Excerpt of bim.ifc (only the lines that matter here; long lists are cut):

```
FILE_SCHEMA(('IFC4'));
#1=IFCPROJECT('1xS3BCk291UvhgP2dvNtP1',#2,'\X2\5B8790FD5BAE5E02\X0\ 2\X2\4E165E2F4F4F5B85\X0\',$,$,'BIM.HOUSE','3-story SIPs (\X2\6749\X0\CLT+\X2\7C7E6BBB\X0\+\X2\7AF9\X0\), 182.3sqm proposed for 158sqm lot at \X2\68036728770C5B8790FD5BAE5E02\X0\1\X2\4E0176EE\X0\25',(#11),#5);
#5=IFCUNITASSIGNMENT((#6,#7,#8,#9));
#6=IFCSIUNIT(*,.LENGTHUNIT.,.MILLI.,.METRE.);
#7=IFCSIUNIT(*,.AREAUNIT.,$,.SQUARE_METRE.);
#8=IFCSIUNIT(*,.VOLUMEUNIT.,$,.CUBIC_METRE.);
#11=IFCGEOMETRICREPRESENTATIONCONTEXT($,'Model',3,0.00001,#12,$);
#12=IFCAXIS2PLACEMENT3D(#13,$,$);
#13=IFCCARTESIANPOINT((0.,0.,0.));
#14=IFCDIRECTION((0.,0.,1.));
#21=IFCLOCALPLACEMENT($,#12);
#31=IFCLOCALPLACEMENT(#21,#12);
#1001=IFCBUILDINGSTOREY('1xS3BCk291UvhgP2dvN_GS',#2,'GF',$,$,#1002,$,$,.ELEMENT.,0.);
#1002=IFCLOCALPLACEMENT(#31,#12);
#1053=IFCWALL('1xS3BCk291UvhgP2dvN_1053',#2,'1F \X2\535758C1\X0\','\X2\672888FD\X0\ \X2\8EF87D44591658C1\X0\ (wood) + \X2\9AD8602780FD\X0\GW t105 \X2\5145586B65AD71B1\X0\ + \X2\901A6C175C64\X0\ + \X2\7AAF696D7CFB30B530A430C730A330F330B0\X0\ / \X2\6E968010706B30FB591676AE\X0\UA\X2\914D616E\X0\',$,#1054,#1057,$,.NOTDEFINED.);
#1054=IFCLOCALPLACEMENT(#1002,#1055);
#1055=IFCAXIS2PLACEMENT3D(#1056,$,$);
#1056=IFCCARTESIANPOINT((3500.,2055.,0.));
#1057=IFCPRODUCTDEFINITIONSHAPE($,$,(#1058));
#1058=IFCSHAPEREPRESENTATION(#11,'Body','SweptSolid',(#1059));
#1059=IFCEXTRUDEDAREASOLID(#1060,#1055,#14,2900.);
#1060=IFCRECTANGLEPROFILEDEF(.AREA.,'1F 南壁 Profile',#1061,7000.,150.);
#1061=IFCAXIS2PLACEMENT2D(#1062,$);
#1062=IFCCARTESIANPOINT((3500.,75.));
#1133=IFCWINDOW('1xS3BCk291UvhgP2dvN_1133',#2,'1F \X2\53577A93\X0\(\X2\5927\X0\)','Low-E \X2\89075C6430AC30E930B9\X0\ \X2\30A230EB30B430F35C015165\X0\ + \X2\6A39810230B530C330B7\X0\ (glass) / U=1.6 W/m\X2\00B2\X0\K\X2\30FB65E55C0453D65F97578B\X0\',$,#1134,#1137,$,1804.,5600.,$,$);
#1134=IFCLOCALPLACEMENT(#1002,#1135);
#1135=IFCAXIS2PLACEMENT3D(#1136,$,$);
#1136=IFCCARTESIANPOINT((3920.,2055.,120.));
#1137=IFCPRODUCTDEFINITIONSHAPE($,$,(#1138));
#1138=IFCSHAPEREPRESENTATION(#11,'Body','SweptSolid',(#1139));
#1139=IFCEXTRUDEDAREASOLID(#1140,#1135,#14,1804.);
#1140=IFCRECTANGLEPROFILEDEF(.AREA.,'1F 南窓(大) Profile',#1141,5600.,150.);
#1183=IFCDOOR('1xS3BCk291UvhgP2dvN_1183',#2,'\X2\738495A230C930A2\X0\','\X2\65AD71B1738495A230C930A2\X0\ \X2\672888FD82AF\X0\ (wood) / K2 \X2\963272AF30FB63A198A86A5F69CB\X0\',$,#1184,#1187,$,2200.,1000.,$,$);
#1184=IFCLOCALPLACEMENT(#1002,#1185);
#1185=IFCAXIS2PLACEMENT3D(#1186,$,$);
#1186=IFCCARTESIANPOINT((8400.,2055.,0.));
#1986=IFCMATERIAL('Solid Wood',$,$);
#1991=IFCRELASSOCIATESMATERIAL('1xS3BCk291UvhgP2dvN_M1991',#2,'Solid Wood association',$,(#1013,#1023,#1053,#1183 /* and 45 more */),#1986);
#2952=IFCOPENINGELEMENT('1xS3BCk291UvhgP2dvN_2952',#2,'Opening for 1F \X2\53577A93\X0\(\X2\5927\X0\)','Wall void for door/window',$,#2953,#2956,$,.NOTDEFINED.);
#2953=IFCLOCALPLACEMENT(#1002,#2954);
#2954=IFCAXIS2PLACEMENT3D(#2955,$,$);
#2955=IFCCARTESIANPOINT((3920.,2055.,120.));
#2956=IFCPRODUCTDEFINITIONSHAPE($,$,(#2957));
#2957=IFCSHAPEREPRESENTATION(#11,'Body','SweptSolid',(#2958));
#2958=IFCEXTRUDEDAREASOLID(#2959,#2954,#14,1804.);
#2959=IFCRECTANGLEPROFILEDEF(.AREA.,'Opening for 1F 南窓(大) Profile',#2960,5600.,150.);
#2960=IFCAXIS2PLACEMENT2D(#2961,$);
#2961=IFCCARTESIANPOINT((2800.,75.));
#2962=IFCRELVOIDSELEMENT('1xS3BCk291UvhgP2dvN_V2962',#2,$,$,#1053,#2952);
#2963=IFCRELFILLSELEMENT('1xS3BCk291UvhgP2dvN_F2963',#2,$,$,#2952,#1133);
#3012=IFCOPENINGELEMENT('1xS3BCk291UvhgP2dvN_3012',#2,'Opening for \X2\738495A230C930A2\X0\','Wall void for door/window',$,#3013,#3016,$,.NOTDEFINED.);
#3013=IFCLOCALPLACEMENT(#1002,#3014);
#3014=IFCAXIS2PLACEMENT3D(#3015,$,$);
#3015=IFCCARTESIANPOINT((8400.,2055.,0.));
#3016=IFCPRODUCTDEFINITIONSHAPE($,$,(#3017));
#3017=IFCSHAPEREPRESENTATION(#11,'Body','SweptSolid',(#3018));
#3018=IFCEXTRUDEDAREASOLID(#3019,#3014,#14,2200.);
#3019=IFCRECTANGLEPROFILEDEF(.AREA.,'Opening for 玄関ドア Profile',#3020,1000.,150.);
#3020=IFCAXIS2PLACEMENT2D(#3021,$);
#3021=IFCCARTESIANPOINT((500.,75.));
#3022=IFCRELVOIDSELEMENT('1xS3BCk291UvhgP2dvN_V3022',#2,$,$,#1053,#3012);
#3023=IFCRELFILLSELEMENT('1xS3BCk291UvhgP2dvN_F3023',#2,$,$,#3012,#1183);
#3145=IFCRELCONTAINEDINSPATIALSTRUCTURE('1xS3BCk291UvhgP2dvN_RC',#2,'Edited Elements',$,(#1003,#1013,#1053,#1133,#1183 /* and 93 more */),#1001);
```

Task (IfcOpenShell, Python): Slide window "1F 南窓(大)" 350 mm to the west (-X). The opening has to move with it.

```python
import ifcopenshell
import ifcopenshell.api.geometry
import ifcopenshell.util.placement
import ifcopenshell.util.unit

model = ifcopenshell.open("bim.ifc")
unit_scale = ifcopenshell.util.unit.calculate_unit_scale(model)

window = model.by_guid("1xS3BCk291UvhgP2dvN_1133")
opening = window.FillsVoids[0].RelatingOpeningElement
wall = opening.VoidsElements[0].RelatingBuildingElement

wall_matrix = ifcopenshell.util.placement.get_local_placement(wall.ObjectPlacement)
shift = wall_matrix[:3, 0] * -0.35 / unit_scale
before = ifcopenshell.util.placement.get_local_placement(window.ObjectPlacement)[:3, 3].copy()

# The window is not placed relative to its opening, so move both.
for product in (opening, window):
    matrix = ifcopenshell.util.placement.get_local_placement(product.ObjectPlacement)
    matrix[:3, 3] += shift
    ifcopenshell.api.geometry.edit_object_placement(model, product=product, matrix=matrix, is_si=False)

after = ifcopenshell.util.placement.get_local_placement(window.ObjectPlacement)[:3, 3]
print("window moved by", (after - before).round(3) + 0.0)

model.write("bim-out.ifc")
```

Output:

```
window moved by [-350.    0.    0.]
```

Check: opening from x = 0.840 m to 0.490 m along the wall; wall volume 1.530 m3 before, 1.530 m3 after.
